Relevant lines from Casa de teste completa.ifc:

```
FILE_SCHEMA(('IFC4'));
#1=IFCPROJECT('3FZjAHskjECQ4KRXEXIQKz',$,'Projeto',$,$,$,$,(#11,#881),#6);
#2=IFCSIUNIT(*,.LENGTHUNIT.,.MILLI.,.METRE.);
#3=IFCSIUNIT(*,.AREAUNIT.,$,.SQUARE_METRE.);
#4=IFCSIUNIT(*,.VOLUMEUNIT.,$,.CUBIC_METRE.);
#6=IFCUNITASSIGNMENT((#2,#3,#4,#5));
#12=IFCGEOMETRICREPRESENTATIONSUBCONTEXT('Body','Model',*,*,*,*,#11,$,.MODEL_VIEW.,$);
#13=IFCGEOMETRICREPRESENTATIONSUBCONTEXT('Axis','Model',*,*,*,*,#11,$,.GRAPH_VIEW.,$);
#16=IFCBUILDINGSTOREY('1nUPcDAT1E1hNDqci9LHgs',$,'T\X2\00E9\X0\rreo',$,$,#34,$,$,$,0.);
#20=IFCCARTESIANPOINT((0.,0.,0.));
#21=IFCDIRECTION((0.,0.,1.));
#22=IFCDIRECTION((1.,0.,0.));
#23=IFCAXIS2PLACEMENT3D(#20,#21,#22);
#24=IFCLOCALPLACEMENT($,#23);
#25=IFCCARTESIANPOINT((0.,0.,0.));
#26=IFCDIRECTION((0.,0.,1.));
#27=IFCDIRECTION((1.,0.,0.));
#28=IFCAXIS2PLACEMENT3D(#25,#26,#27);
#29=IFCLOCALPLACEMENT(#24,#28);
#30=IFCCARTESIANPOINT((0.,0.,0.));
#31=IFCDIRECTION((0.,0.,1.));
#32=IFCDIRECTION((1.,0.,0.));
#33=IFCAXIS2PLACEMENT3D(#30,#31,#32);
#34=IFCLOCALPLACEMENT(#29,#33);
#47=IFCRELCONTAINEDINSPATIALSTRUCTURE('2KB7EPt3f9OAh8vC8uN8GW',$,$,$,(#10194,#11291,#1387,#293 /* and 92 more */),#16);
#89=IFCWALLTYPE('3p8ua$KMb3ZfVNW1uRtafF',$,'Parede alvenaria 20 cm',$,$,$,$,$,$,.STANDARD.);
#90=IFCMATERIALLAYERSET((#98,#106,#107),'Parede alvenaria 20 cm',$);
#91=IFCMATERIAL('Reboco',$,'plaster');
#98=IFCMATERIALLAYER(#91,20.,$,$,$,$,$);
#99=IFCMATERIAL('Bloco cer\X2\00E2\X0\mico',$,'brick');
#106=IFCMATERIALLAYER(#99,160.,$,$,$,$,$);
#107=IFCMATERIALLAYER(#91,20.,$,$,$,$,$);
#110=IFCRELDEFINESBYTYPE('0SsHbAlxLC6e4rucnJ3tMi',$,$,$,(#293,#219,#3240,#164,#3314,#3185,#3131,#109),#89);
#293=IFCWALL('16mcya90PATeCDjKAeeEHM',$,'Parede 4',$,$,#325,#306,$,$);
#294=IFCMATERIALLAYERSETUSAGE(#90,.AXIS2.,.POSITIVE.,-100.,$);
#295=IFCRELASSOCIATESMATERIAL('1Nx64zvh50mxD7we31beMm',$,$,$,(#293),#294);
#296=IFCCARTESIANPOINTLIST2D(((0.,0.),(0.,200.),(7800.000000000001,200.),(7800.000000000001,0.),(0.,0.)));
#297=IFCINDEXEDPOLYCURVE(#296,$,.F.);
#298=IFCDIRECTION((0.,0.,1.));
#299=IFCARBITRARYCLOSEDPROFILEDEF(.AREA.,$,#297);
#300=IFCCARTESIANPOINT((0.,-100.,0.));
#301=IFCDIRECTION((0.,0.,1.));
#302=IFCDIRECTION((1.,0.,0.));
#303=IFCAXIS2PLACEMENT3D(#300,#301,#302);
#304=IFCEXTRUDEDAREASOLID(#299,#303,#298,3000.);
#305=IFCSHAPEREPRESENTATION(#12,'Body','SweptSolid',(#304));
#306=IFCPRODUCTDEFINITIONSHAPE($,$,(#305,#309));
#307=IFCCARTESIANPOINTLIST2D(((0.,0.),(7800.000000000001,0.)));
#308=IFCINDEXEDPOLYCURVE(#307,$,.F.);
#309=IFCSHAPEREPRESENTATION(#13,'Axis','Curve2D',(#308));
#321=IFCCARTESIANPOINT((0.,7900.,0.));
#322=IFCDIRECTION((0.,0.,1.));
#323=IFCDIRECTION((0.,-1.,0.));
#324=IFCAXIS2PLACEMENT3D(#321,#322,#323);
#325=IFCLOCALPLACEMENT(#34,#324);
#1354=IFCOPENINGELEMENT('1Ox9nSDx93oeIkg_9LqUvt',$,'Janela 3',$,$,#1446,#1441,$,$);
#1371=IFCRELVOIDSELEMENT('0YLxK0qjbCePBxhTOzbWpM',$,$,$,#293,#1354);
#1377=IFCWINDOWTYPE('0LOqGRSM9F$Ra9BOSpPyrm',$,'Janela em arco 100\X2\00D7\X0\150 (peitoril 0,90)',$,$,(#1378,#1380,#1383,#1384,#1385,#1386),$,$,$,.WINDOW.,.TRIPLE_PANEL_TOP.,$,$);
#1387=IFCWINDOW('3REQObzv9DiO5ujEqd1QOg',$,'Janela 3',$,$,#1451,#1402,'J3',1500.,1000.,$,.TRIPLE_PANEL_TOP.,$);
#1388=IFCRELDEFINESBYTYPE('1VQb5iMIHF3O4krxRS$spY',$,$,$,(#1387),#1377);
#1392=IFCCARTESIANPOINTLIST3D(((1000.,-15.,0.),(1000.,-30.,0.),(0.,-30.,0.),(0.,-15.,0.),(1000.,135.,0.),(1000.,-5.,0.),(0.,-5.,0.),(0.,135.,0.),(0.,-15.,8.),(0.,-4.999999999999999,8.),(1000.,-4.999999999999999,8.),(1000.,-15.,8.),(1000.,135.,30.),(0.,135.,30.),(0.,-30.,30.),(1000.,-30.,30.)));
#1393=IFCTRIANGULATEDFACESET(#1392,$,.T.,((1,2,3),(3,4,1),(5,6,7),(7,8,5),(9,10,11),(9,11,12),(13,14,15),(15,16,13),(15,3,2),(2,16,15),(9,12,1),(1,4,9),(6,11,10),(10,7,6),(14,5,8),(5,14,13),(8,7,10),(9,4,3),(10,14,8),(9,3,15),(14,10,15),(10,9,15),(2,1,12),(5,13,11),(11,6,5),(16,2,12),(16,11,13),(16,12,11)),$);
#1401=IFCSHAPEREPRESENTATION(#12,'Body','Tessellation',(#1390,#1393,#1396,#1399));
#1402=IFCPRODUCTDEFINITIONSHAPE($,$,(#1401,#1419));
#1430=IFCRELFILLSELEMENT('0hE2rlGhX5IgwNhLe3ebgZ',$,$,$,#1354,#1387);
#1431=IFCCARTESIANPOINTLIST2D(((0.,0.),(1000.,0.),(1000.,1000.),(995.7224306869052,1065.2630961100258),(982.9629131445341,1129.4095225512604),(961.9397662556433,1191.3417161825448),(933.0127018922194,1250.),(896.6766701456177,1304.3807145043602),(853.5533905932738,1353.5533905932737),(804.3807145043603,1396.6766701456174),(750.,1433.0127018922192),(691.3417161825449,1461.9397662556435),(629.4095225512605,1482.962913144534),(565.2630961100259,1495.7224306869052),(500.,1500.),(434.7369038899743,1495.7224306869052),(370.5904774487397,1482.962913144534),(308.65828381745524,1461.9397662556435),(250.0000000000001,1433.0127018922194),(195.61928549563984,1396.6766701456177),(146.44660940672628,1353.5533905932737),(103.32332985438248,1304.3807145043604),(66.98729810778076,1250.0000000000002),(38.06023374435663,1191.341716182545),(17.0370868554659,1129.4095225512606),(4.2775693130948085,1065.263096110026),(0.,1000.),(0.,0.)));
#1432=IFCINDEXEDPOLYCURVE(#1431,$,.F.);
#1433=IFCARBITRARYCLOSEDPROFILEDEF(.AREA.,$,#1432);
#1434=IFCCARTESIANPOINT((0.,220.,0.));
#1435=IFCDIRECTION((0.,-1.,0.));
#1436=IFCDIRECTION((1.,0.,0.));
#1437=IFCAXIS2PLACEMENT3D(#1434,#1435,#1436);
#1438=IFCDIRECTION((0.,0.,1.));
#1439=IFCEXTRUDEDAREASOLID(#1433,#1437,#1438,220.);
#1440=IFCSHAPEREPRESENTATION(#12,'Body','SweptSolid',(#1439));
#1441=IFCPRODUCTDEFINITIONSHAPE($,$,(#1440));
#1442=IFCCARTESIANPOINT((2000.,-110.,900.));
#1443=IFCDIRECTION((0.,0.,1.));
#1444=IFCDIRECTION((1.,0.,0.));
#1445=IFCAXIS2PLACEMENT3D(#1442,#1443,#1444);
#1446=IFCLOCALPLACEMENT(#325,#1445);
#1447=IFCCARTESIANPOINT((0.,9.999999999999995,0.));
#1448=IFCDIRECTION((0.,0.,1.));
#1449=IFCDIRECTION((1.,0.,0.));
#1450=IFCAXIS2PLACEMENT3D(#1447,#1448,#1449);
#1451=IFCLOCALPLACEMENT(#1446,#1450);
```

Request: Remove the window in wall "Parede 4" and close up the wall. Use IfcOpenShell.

```python
import ifcopenshell
import ifcopenshell.api.feature
import ifcopenshell.api.root
import ifcopenshell.geom
import ifcopenshell.util.shape

model = ifcopenshell.open("Casa de teste completa.ifc")
settings = ifcopenshell.geom.settings()


def volume(element):
    """Net volume in cubic metres, openings subtracted."""
    shape = ifcopenshell.geom.create_shape(settings, element)
    return ifcopenshell.util.shape.get_volume(shape.geometry)


window = model.by_guid("3REQObzv9DiO5ujEqd1QOg")
opening = window.FillsVoids[0].RelatingOpeningElement
wall = opening.VoidsElements[0].RelatingBuildingElement
before = volume(wall)

ifcopenshell.api.root.remove_product(model, product=window)
ifcopenshell.api.feature.remove_feature(model, feature=opening)

after = volume(wall)

print(f"wall volume {before:.3f} -> {after:.3f} m3")

model.write("Casa de teste completa_updated.ifc")
```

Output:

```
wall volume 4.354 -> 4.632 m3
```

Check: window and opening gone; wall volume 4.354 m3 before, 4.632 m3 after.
